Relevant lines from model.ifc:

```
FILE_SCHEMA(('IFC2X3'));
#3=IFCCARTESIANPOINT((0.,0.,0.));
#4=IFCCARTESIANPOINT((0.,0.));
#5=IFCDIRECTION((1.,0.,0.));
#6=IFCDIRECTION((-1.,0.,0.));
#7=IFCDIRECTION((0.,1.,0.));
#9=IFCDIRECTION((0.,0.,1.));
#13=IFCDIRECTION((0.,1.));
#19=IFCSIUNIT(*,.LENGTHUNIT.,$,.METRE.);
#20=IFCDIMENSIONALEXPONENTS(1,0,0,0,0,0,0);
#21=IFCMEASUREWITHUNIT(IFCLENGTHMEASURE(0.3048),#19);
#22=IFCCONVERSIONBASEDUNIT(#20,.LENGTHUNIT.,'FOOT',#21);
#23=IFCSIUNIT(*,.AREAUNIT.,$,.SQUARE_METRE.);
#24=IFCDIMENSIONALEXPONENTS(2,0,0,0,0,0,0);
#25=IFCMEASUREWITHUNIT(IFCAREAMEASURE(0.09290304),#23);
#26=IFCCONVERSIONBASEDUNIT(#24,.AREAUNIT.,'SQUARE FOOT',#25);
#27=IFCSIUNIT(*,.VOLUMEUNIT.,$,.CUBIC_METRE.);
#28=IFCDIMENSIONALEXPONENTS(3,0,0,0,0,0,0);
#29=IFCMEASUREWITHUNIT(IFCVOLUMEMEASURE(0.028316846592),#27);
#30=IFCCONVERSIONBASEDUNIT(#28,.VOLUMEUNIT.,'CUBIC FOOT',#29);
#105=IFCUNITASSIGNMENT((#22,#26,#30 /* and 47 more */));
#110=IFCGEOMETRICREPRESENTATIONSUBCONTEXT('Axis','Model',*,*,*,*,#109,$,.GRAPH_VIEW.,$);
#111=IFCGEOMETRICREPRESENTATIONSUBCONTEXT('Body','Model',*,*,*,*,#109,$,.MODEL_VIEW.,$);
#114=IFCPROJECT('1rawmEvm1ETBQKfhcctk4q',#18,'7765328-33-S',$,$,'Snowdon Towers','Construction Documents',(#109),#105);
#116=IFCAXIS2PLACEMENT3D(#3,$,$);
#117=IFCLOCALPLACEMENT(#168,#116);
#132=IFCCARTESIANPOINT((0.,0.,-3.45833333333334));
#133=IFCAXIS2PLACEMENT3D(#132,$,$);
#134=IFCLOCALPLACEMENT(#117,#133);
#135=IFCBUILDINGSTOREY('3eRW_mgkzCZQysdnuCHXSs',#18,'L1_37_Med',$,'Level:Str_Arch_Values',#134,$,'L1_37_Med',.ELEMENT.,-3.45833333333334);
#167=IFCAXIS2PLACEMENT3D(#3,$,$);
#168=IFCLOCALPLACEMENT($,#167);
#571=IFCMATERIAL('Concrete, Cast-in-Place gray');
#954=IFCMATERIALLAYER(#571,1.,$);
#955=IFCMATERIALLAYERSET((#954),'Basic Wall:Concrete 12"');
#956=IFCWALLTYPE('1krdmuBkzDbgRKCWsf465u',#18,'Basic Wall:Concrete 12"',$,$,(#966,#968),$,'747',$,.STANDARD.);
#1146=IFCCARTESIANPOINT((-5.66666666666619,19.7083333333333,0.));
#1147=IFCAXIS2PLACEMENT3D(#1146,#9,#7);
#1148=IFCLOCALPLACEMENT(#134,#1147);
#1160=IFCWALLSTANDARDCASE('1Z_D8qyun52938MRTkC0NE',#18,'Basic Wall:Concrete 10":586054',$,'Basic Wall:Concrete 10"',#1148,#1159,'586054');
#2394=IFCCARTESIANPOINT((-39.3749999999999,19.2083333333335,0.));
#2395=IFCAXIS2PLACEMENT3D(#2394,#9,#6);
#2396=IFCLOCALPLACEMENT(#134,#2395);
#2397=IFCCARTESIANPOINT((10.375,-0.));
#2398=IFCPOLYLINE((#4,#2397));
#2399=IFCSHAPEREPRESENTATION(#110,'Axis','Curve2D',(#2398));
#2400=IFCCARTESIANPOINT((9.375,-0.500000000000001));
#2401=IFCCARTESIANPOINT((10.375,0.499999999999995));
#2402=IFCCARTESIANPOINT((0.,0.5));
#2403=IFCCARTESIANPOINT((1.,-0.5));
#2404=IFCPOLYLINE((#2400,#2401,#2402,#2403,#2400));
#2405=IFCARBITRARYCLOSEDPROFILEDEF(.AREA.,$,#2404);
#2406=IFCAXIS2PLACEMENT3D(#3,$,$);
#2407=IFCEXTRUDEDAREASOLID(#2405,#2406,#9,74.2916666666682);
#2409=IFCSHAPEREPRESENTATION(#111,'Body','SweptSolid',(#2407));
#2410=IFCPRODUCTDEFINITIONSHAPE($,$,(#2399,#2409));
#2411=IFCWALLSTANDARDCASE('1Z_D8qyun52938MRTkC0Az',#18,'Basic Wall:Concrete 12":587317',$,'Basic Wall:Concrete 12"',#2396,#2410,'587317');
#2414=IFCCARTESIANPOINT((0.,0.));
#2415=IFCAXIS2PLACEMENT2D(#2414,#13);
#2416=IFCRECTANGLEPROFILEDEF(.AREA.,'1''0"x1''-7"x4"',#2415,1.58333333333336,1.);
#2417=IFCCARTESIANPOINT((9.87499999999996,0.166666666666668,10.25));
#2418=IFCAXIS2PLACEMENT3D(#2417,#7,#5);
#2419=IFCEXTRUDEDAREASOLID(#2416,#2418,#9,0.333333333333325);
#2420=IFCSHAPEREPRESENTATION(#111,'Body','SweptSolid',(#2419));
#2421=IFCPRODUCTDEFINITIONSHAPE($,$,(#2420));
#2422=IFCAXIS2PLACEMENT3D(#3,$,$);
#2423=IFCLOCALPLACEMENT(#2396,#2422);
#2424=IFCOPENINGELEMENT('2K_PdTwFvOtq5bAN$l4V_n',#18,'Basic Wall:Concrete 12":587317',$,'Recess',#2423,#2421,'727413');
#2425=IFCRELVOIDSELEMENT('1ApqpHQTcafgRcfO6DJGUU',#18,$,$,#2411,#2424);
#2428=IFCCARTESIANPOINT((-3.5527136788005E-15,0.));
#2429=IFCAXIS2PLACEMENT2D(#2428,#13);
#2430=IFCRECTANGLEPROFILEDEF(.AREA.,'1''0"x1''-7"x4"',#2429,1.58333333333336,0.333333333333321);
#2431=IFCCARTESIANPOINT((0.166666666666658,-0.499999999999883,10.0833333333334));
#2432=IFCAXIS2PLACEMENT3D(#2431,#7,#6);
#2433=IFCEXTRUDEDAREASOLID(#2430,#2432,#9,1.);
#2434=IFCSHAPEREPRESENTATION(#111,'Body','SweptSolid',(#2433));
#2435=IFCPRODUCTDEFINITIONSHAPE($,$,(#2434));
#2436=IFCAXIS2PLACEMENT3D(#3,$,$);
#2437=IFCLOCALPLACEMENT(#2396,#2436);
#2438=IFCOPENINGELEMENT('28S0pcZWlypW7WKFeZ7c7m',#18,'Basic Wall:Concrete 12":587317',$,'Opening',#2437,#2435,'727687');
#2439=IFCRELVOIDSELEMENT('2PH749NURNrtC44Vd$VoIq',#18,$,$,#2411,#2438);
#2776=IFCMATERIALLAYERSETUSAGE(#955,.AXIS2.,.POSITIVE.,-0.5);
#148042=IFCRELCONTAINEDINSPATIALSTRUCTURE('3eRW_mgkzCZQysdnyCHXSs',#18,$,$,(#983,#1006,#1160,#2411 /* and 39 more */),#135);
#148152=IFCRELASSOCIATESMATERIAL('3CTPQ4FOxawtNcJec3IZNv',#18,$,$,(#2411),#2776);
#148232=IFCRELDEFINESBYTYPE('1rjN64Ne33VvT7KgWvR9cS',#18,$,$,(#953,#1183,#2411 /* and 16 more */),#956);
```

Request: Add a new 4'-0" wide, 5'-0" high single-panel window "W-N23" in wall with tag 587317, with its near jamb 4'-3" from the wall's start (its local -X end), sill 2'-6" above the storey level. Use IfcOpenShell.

```python
import numpy as np
import ifcopenshell
import ifcopenshell.api.feature
import ifcopenshell.api.geometry
import ifcopenshell.api.root
import ifcopenshell.api.spatial
import ifcopenshell.api.type
import ifcopenshell.geom
import ifcopenshell.util.element
import ifcopenshell.util.placement
import ifcopenshell.util.representation
import ifcopenshell.util.shape
import ifcopenshell.util.unit

model = ifcopenshell.open("model.ifc")
unit_scale = ifcopenshell.util.unit.calculate_unit_scale(model)
settings = ifcopenshell.geom.settings()


def volume(element):
    """Net volume in cubic metres, openings subtracted."""
    shape = ifcopenshell.geom.create_shape(settings, element)
    return ifcopenshell.util.shape.get_volume(shape.geometry)


wall = model.by_guid("1Z_D8qyun52938MRTkC0Az")
storey = ifcopenshell.util.element.get_container(wall, ifc_class="IfcBuildingStorey")
context = ifcopenshell.util.representation.get_context(model, "Model", "Body", "MODEL_VIEW")
before = volume(wall)

width, height, from_end, sill = 1.2192, 1.524, 1.2954, 0.762  # metres

# The wall runs along its own X axis, and the end named is its -X end.
wall_shape = ifcopenshell.geom.create_shape(settings, wall)
x, y, z = ifcopenshell.util.shape.get_vertices(wall_shape.geometry).T
start = x.min() + from_end
face, thickness = float(y.min()), float(y.max() - y.min())
wall_matrix = ifcopenshell.util.placement.get_local_placement(wall.ObjectPlacement)
level = ifcopenshell.util.placement.get_local_placement(storey.ObjectPlacement)[2, 3]


def in_wall(x, y):
    """Placement at x, y metres in the wall's axes, at sill height."""
    matrix = wall_matrix.copy()
    matrix[:, 3] = wall_matrix @ np.array([x / unit_scale, y / unit_scale, 0.0, 1.0])
    matrix[2, 3] = level + sill / unit_scale
    return matrix


# Opening: a box that overshoots both wall faces by 50 mm.
opening = ifcopenshell.api.root.create_entity(model, ifc_class="IfcOpeningElement")
box = ifcopenshell.api.geometry.add_wall_representation(
    model, context=context, length=width, height=height, thickness=thickness + 0.1
)
ifcopenshell.api.geometry.assign_representation(model, product=opening, representation=box)
ifcopenshell.api.geometry.edit_object_placement(model, product=opening, matrix=in_wall(start, face - 0.05), is_si=False)
ifcopenshell.api.feature.add_feature(model, feature=opening, element=wall)

window = ifcopenshell.api.root.create_entity(model, ifc_class="IfcWindow", name="W-N23")
window.OverallWidth, window.OverallHeight = width / unit_scale, height / unit_scale
body = ifcopenshell.api.geometry.add_window_representation(
    model,
    context=context,
    overall_width=window.OverallWidth,
    overall_height=window.OverallHeight,
    partition_type="SINGLE_PANEL",
)
ifcopenshell.api.geometry.assign_representation(model, product=window, representation=body)
ifcopenshell.api.spatial.assign_container(model, products=[window], relating_structure=storey)
fills = ifcopenshell.api.feature.add_filling(model, opening=opening, element=window)
fills.OwnerHistory = window.OwnerHistory  # required in IFC2X3

# IFC2X3 keeps the operation on the window style.
style = ifcopenshell.api.root.create_entity(model, ifc_class="IfcWindowStyle", name="W-N23")
style.OperationType, style.ConstructionType = "SINGLE_PANEL", "NOTDEFINED"
style.ParameterTakesPrecedence = style.Sizeable = False
ifcopenshell.api.type.assign_type(model, related_objects=[window], relating_type=style)

# Centre the window in the wall's thickness.
ifcopenshell.api.geometry.edit_object_placement(model, product=window, matrix=in_wall(start, face), is_si=False)
window_shape = ifcopenshell.geom.create_shape(settings, window)
depth = ifcopenshell.util.shape.get_vertices(window_shape.geometry)[:, 1]
offset = face + thickness / 2 - (depth.min() + depth.max()) / 2
ifcopenshell.api.geometry.edit_object_placement(model, product=window, matrix=in_wall(start, offset), is_si=False)

after = volume(wall)

print(f"wall volume {before:.3f} -> {after:.3f} m3")

model.write("model_edited.ifc")
```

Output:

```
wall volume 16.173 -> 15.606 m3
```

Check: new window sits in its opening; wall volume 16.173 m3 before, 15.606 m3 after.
